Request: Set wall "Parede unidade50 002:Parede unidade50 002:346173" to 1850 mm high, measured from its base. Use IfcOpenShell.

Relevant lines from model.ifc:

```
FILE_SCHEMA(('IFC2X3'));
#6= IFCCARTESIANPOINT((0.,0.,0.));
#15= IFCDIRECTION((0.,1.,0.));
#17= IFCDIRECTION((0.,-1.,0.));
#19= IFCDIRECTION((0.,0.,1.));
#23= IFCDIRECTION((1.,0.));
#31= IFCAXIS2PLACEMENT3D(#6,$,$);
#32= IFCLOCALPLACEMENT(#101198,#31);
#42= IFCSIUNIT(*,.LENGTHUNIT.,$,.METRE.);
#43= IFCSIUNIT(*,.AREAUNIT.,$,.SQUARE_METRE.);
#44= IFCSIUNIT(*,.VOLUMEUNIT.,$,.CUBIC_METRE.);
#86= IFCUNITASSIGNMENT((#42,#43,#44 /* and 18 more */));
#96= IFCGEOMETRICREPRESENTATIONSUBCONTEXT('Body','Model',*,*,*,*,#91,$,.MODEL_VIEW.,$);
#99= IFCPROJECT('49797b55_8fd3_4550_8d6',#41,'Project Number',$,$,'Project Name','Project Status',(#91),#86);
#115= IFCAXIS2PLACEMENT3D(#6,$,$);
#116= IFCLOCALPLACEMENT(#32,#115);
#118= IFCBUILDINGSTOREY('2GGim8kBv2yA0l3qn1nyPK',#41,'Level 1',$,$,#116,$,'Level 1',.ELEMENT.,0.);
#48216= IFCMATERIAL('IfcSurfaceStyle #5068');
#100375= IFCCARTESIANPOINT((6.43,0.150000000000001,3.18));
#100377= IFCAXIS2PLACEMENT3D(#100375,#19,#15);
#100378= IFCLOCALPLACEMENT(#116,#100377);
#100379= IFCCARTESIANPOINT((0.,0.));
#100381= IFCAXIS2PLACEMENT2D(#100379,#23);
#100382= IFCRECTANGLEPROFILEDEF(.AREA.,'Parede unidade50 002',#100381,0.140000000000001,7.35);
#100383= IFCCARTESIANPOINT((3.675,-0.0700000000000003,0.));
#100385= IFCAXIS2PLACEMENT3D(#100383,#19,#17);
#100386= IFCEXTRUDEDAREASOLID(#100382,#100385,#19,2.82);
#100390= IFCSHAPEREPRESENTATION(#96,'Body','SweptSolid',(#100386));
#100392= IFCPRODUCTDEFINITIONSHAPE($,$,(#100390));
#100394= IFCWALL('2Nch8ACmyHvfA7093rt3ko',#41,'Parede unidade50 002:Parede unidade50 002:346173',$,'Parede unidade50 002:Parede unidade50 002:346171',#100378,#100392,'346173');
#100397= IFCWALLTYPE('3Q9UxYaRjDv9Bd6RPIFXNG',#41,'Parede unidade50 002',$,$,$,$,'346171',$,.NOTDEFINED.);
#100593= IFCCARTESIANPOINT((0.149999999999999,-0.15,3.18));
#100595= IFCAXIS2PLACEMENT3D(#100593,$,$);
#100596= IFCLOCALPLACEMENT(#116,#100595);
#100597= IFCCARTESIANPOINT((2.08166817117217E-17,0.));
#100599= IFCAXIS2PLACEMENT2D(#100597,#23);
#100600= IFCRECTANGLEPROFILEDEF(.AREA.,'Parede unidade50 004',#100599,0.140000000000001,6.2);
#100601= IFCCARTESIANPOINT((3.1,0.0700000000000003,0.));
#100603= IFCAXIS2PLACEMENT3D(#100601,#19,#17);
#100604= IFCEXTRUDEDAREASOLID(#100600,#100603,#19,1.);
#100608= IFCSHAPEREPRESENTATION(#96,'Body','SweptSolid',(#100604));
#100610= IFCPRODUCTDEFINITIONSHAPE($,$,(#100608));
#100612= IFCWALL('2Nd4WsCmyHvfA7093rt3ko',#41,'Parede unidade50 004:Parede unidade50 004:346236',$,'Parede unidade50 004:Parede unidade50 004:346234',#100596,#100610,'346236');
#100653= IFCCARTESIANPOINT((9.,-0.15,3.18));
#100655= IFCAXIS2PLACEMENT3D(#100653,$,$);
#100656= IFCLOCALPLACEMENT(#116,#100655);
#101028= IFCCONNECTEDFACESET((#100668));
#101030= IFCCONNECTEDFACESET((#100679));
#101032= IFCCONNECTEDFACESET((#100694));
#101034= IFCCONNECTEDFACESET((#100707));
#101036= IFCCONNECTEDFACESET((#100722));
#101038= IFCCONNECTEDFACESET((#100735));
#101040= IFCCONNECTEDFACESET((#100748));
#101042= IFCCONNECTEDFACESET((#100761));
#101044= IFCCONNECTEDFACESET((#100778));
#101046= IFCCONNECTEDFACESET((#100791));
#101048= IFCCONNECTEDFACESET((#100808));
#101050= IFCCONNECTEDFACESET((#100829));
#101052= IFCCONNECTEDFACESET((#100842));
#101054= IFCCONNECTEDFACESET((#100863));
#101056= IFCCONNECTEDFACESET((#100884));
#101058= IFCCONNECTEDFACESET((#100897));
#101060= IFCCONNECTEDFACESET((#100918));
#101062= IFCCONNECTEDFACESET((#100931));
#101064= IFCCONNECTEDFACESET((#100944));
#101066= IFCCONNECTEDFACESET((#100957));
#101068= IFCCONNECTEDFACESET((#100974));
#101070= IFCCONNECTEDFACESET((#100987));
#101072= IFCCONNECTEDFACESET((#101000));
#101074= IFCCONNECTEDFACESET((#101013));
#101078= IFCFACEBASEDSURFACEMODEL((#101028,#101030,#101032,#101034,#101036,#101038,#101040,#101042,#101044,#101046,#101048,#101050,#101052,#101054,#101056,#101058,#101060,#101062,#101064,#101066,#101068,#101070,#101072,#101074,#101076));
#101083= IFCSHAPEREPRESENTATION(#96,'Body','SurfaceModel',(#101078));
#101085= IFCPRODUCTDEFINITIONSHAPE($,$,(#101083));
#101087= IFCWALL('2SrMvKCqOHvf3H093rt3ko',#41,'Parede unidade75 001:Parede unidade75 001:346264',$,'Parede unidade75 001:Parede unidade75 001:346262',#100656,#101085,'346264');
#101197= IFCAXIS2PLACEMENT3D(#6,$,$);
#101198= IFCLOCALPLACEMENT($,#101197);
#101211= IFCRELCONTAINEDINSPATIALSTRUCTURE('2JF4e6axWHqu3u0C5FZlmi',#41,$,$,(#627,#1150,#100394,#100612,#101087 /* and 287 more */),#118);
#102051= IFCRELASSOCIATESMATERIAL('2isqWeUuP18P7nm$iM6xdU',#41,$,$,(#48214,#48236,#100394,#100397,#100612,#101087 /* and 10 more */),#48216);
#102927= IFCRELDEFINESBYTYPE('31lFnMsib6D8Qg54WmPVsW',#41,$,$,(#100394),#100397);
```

```python
import ifcopenshell
import ifcopenshell.geom
import ifcopenshell.util.representation
import ifcopenshell.util.shape
import ifcopenshell.util.unit

model = ifcopenshell.open("model.ifc")
unit_scale = ifcopenshell.util.unit.calculate_unit_scale(model)
settings = ifcopenshell.geom.settings()


def volume(element):
    """Net volume in cubic metres, openings subtracted."""
    shape = ifcopenshell.geom.create_shape(settings, element)
    return ifcopenshell.util.shape.get_volume(shape.geometry)


wall = model.by_guid("2Nch8ACmyHvfA7093rt3ko")
before = volume(wall)

body = ifcopenshell.util.representation.get_representation(wall, "Model", "Body")
solid = body.Items[0]
old_height = solid.Depth
solid.Depth = 1.85 / unit_scale
after = volume(wall)

print(f"height {old_height:g} -> {solid.Depth:g}, volume {before:.3f} -> {after:.3f} m3")

model.write("model_v2.ifc")
```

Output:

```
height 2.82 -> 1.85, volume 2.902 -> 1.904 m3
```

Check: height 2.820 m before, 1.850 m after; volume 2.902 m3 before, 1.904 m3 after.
